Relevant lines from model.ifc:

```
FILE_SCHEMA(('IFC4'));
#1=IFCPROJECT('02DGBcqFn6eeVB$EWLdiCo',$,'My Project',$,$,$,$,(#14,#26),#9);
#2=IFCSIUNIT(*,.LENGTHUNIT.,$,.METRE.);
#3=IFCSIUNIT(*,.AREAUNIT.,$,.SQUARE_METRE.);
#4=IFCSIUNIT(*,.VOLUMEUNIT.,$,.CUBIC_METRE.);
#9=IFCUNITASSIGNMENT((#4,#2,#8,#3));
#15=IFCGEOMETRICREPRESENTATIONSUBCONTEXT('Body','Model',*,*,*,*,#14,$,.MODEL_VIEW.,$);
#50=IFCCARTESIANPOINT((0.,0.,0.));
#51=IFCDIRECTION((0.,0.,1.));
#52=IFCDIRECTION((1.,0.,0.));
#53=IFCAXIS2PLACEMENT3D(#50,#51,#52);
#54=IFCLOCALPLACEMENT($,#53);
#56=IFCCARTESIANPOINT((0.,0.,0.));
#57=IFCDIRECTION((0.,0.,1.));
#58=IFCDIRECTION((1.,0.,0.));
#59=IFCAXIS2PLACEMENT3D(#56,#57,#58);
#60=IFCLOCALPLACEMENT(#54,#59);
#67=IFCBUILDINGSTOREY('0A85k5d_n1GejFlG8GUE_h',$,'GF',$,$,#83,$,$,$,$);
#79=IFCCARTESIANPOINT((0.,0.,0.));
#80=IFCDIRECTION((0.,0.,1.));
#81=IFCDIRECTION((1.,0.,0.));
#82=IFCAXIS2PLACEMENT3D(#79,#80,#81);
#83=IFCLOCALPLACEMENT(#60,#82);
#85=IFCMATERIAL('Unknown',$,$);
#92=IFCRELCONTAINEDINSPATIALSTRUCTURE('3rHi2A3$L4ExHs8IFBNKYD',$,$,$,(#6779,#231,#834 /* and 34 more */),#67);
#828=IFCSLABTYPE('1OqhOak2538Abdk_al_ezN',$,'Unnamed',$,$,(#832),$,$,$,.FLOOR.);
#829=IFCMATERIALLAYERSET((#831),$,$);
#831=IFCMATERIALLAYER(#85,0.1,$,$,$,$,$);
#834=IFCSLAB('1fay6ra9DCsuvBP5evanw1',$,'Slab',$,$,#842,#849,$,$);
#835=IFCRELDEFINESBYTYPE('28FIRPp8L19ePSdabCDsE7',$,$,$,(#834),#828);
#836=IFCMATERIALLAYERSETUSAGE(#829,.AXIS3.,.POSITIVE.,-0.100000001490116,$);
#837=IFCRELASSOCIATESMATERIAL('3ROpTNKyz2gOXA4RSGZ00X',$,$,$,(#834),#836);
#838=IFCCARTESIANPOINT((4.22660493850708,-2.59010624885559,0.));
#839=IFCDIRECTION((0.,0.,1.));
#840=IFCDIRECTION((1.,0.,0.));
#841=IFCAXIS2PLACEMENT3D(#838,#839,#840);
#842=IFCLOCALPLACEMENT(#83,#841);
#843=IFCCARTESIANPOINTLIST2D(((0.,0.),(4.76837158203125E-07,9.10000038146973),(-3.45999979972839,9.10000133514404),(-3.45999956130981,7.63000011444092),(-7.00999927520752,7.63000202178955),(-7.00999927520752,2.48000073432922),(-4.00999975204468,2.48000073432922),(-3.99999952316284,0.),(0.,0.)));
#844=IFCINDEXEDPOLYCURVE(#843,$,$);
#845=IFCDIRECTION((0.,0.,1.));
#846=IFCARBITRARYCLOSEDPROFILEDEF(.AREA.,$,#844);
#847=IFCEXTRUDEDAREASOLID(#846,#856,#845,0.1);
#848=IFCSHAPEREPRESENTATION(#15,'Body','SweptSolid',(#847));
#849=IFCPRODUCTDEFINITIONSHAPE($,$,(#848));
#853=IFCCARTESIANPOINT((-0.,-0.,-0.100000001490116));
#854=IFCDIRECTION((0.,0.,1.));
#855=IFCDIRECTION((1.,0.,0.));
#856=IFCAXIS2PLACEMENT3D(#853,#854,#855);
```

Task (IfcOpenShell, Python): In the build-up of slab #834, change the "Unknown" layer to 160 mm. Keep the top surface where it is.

```python
import ifcopenshell
import ifcopenshell.util.element
import ifcopenshell.util.representation

model = ifcopenshell.open("model.ifc")

layer_set = model.by_id(829)
layer = next(l for l in layer_set.MaterialLayers if l.Material and l.Material.Name == "Unknown")
change = 0.16 - layer.LayerThickness
layer.LayerThickness += change

# Geometry does not follow the layer set by itself.
slabs = [e for e in ifcopenshell.util.element.get_elements_by_material(model, layer_set) if e.is_a("IfcSlab")]
for slab in sorted(slabs, key=lambda e: e.id()):
    body = ifcopenshell.util.representation.get_representation(slab, "Model", "Body")
    solid = body.Items[0]
    old_depth = solid.Depth
    solid.Depth += change
    # Extruded upwards: lower the start of the extrusion so the top stays.
    x, y, z = solid.Position.Location.Coordinates
    solid.Position.Location = model.createIfcCartesianPoint((x, y, z - change))
    print(slab.id(), f"{old_depth:g} -> {solid.Depth:g}")

# The layers are counted up from the underside, which has moved.
for usage in {ifcopenshell.util.element.get_material(slab) for slab in slabs}:
    usage.OffsetFromReferenceLine -= change

model.write("model_v2.ifc")
```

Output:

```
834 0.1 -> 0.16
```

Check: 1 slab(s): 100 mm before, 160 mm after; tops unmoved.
